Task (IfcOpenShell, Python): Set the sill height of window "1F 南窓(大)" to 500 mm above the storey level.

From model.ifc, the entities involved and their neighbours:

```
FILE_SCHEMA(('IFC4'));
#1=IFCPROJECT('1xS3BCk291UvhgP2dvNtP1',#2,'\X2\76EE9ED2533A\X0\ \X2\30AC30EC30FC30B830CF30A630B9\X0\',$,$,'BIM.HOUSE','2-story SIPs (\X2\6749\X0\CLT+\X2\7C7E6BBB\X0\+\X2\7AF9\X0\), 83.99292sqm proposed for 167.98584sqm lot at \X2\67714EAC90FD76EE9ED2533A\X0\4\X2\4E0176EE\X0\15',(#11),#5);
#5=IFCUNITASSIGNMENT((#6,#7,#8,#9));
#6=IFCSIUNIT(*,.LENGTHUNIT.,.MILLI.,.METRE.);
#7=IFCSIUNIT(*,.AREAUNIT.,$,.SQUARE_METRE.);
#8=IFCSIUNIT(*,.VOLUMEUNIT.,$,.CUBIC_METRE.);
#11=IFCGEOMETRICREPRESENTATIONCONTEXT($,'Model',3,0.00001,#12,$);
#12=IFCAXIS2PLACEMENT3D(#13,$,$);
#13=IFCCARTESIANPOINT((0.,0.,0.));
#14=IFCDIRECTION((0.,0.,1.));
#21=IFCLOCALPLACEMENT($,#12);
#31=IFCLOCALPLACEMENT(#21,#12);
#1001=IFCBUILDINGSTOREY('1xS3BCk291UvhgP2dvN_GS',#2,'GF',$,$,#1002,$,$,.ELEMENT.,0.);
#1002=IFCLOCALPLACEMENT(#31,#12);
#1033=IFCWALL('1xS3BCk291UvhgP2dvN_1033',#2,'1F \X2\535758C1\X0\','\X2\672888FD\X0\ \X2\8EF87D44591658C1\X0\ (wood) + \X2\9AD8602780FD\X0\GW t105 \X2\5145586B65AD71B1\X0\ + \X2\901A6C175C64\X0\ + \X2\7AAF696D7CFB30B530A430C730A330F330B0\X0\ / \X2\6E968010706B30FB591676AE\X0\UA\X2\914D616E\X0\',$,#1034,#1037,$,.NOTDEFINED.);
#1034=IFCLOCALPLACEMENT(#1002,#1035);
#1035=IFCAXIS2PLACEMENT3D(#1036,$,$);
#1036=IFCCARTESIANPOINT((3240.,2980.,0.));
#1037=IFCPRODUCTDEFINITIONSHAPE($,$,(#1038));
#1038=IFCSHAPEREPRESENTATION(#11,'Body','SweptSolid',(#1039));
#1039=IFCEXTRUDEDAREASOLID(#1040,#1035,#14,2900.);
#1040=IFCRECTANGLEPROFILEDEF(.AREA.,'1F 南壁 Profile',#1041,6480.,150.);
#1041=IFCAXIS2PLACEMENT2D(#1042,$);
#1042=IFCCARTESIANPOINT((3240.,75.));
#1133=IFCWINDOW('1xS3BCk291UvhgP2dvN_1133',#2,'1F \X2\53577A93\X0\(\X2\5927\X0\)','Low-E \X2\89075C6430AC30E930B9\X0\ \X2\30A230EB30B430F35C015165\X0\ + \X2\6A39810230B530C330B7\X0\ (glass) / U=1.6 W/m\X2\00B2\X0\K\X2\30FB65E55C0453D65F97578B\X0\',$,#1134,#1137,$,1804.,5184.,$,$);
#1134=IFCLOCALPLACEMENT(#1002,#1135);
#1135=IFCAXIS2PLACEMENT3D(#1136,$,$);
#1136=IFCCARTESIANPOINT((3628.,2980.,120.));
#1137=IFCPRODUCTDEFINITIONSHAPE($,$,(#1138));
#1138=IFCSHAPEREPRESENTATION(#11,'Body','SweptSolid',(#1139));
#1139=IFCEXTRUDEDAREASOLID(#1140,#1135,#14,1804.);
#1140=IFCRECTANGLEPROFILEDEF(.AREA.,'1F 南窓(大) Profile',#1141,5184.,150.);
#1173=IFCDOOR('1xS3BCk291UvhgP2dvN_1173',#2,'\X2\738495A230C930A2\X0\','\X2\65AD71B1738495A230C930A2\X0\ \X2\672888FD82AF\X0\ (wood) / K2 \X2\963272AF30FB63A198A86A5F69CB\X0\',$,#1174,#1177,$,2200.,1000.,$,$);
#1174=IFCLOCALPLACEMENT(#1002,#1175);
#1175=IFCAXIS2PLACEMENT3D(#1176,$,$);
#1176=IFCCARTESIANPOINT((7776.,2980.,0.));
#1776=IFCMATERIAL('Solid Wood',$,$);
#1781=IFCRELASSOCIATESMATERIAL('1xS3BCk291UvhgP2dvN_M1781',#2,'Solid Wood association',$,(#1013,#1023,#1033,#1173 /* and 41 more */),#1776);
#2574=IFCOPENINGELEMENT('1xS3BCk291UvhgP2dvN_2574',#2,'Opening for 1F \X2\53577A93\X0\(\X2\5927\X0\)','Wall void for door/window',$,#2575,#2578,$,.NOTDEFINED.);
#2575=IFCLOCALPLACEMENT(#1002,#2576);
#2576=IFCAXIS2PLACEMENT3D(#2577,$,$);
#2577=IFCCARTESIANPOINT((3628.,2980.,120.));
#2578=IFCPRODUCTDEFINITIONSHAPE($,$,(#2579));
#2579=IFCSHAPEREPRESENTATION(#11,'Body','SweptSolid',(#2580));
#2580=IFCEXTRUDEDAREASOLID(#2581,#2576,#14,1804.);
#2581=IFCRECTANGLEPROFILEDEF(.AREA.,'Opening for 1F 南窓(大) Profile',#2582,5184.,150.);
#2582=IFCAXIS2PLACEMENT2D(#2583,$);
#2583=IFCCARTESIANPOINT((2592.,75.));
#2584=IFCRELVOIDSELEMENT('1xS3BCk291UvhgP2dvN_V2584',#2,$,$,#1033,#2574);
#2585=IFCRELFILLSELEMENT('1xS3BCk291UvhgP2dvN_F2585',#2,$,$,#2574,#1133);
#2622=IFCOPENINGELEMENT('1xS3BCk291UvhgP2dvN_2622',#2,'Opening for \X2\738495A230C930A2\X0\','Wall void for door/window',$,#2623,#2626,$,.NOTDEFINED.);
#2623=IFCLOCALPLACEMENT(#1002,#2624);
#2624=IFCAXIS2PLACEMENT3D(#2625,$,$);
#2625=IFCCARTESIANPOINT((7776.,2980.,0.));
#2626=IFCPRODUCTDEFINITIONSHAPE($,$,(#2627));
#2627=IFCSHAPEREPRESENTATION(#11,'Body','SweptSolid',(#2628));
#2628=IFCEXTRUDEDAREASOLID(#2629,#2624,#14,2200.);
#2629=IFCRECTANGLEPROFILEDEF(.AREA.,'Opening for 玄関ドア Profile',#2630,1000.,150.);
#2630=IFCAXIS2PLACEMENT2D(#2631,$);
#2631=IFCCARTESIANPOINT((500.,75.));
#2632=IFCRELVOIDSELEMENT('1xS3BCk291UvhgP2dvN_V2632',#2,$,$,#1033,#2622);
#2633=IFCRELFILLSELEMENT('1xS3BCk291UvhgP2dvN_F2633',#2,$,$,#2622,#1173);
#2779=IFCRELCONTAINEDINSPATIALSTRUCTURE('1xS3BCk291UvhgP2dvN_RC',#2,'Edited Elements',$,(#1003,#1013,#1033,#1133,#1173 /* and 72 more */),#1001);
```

```python
import numpy as np
import ifcopenshell
import ifcopenshell.api.geometry
import ifcopenshell.geom
import ifcopenshell.util.element
import ifcopenshell.util.placement
import ifcopenshell.util.shape
import ifcopenshell.util.unit

model = ifcopenshell.open("model.ifc")
unit_scale = ifcopenshell.util.unit.calculate_unit_scale(model)

window = model.by_guid("1xS3BCk291UvhgP2dvN_1133")
opening = window.FillsVoids[0].RelatingOpeningElement
storey = ifcopenshell.util.element.get_container(window, ifc_class="IfcBuildingStorey")
level = ifcopenshell.util.placement.get_local_placement(storey.ObjectPlacement)[2, 3]

# The opening's origin need not be at the sill, so measure its lowest point.
shape = ifcopenshell.geom.create_shape(ifcopenshell.geom.settings(), opening)
bottom = ifcopenshell.util.shape.get_shape_bottom_elevation(shape, shape.geometry) / unit_scale
dz = level + 500.0 - bottom

shift = np.array([0.0, 0.0, dz])
# The window is not placed relative to its opening, so move both.
for product in (opening, window):
    matrix = ifcopenshell.util.placement.get_local_placement(product.ObjectPlacement)
    matrix[:3, 3] += shift
    ifcopenshell.api.geometry.edit_object_placement(model, product=product, matrix=matrix, is_si=False)

print(f"moved by {dz * unit_scale:+.3f} m")

model.write("model_v2.ifc")
```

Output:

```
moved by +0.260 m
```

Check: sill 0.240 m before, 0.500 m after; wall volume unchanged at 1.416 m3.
